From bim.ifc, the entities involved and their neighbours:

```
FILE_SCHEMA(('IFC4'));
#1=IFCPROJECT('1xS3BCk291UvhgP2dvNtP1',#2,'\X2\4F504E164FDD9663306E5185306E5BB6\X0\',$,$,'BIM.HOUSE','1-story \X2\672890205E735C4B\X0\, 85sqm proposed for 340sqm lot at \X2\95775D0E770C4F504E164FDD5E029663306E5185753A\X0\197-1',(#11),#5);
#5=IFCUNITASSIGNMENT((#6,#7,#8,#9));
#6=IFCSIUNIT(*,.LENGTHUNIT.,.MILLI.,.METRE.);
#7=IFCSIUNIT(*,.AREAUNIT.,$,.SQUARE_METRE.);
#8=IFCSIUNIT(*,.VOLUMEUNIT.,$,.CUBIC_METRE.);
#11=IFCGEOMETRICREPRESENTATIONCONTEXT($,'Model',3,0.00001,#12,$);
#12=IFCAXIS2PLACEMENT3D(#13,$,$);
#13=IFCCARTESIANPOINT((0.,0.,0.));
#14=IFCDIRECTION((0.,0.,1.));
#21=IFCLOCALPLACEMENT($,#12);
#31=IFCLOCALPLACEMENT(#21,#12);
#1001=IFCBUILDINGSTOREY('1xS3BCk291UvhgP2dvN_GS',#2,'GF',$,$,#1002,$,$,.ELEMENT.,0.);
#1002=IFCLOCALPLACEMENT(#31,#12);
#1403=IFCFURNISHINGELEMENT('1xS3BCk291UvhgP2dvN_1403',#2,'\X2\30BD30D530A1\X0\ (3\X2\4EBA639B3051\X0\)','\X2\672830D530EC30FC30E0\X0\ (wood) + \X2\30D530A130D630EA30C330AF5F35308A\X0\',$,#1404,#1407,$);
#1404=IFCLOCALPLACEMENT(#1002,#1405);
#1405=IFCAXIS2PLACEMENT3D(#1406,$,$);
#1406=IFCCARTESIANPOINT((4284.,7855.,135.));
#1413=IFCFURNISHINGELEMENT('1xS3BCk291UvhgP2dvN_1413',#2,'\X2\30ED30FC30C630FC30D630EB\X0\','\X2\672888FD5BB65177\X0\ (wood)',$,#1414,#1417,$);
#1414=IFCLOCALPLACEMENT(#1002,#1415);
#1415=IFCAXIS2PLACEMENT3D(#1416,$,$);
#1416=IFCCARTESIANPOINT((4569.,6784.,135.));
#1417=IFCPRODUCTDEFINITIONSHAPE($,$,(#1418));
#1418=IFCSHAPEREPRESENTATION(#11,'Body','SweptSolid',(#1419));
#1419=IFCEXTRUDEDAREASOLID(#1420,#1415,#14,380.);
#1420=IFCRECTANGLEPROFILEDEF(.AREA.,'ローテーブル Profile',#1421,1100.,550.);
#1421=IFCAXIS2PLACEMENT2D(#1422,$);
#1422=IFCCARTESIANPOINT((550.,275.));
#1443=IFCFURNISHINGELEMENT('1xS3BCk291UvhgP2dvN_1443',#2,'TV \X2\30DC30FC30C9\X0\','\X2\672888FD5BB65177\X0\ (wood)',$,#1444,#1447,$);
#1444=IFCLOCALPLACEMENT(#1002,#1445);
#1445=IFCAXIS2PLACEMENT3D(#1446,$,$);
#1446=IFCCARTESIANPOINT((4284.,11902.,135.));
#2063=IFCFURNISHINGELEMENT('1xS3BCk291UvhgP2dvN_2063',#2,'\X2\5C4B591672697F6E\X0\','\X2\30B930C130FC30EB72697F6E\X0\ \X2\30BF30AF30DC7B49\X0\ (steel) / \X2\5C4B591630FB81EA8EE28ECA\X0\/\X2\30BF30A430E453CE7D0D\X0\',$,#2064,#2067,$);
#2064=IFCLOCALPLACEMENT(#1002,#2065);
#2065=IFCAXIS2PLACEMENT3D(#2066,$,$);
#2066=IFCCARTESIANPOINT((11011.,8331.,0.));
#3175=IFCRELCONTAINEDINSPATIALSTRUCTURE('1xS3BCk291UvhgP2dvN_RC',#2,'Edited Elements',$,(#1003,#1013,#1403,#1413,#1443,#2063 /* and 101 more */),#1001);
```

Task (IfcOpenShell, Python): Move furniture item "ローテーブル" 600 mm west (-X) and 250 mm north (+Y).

```python
import ifcopenshell
import ifcopenshell.api.geometry
import ifcopenshell.util.placement
import ifcopenshell.util.unit

model = ifcopenshell.open("bim.ifc")
unit_scale = ifcopenshell.util.unit.calculate_unit_scale(model)

item = model.by_guid("1xS3BCk291UvhgP2dvN_1413")
matrix = ifcopenshell.util.placement.get_local_placement(item.ObjectPlacement)
matrix[0, 3] -= 0.6 / unit_scale
matrix[1, 3] += 0.25 / unit_scale
ifcopenshell.api.geometry.edit_object_placement(model, product=item, matrix=matrix, is_si=False)

print(ifcopenshell.util.placement.get_local_placement(item.ObjectPlacement).round(3) + 0.0)

model.write("bim_rev.ifc")
```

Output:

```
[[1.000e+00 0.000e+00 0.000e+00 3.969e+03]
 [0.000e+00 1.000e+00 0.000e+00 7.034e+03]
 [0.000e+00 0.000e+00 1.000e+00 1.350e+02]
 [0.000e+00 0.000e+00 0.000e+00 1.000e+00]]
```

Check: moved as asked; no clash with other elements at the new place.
